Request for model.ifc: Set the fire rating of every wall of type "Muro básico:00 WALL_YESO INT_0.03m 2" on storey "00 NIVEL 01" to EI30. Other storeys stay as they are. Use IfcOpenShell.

First a look at what the model holds.

```python
import ifcopenshell
import ifcopenshell.util.element

model = ifcopenshell.open("model.ifc")
print(model.schema)
storey = next(s for s in model.by_type("IfcBuildingStorey") if s.Name == "00 NIVEL 01")
walls = [e for e in ifcopenshell.util.element.get_decomposition(storey) if e.is_a("IfcWall")]
seen = {}
for e in walls:
    element_type = ifcopenshell.util.element.get_type(e)
    key = (element_type.Name if element_type != e and element_type else None, ifcopenshell.util.element.get_pset(e, "Pset_WallCommon", "FireRating"))
    seen[key] = seen.get(key, 0) + 1
for (name, value), count in sorted(seen.items(), key=str):
    print(count, "x", name, "|", value)
```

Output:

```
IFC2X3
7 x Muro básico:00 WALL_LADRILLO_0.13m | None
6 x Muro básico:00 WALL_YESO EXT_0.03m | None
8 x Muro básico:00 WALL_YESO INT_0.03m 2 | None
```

```python
import ifcopenshell
import ifcopenshell.api.pset
import ifcopenshell.util.element

model = ifcopenshell.open("model.ifc")

storey = next(s for s in model.by_type("IfcBuildingStorey") if s.Name == "00 NIVEL 01")
walls = [e for e in ifcopenshell.util.element.get_decomposition(storey) if e.is_a("IfcWall")]

count = 0
for e in walls:
    element_type = ifcopenshell.util.element.get_type(e)
    if element_type in (None, e) or element_type.Name != "Muro básico:00 WALL_YESO INT_0.03m 2":
        continue
    # add_pset returns the element's existing set when there is one.
    pset = ifcopenshell.api.pset.add_pset(model, product=e, name="Pset_WallCommon")
    ifcopenshell.api.pset.edit_pset(model, pset=pset, properties={"FireRating": "EI30"})
    count += 1

print(count, "walls updated")

model.write("model_edited.ifc")
```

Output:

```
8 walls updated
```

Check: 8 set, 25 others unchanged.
